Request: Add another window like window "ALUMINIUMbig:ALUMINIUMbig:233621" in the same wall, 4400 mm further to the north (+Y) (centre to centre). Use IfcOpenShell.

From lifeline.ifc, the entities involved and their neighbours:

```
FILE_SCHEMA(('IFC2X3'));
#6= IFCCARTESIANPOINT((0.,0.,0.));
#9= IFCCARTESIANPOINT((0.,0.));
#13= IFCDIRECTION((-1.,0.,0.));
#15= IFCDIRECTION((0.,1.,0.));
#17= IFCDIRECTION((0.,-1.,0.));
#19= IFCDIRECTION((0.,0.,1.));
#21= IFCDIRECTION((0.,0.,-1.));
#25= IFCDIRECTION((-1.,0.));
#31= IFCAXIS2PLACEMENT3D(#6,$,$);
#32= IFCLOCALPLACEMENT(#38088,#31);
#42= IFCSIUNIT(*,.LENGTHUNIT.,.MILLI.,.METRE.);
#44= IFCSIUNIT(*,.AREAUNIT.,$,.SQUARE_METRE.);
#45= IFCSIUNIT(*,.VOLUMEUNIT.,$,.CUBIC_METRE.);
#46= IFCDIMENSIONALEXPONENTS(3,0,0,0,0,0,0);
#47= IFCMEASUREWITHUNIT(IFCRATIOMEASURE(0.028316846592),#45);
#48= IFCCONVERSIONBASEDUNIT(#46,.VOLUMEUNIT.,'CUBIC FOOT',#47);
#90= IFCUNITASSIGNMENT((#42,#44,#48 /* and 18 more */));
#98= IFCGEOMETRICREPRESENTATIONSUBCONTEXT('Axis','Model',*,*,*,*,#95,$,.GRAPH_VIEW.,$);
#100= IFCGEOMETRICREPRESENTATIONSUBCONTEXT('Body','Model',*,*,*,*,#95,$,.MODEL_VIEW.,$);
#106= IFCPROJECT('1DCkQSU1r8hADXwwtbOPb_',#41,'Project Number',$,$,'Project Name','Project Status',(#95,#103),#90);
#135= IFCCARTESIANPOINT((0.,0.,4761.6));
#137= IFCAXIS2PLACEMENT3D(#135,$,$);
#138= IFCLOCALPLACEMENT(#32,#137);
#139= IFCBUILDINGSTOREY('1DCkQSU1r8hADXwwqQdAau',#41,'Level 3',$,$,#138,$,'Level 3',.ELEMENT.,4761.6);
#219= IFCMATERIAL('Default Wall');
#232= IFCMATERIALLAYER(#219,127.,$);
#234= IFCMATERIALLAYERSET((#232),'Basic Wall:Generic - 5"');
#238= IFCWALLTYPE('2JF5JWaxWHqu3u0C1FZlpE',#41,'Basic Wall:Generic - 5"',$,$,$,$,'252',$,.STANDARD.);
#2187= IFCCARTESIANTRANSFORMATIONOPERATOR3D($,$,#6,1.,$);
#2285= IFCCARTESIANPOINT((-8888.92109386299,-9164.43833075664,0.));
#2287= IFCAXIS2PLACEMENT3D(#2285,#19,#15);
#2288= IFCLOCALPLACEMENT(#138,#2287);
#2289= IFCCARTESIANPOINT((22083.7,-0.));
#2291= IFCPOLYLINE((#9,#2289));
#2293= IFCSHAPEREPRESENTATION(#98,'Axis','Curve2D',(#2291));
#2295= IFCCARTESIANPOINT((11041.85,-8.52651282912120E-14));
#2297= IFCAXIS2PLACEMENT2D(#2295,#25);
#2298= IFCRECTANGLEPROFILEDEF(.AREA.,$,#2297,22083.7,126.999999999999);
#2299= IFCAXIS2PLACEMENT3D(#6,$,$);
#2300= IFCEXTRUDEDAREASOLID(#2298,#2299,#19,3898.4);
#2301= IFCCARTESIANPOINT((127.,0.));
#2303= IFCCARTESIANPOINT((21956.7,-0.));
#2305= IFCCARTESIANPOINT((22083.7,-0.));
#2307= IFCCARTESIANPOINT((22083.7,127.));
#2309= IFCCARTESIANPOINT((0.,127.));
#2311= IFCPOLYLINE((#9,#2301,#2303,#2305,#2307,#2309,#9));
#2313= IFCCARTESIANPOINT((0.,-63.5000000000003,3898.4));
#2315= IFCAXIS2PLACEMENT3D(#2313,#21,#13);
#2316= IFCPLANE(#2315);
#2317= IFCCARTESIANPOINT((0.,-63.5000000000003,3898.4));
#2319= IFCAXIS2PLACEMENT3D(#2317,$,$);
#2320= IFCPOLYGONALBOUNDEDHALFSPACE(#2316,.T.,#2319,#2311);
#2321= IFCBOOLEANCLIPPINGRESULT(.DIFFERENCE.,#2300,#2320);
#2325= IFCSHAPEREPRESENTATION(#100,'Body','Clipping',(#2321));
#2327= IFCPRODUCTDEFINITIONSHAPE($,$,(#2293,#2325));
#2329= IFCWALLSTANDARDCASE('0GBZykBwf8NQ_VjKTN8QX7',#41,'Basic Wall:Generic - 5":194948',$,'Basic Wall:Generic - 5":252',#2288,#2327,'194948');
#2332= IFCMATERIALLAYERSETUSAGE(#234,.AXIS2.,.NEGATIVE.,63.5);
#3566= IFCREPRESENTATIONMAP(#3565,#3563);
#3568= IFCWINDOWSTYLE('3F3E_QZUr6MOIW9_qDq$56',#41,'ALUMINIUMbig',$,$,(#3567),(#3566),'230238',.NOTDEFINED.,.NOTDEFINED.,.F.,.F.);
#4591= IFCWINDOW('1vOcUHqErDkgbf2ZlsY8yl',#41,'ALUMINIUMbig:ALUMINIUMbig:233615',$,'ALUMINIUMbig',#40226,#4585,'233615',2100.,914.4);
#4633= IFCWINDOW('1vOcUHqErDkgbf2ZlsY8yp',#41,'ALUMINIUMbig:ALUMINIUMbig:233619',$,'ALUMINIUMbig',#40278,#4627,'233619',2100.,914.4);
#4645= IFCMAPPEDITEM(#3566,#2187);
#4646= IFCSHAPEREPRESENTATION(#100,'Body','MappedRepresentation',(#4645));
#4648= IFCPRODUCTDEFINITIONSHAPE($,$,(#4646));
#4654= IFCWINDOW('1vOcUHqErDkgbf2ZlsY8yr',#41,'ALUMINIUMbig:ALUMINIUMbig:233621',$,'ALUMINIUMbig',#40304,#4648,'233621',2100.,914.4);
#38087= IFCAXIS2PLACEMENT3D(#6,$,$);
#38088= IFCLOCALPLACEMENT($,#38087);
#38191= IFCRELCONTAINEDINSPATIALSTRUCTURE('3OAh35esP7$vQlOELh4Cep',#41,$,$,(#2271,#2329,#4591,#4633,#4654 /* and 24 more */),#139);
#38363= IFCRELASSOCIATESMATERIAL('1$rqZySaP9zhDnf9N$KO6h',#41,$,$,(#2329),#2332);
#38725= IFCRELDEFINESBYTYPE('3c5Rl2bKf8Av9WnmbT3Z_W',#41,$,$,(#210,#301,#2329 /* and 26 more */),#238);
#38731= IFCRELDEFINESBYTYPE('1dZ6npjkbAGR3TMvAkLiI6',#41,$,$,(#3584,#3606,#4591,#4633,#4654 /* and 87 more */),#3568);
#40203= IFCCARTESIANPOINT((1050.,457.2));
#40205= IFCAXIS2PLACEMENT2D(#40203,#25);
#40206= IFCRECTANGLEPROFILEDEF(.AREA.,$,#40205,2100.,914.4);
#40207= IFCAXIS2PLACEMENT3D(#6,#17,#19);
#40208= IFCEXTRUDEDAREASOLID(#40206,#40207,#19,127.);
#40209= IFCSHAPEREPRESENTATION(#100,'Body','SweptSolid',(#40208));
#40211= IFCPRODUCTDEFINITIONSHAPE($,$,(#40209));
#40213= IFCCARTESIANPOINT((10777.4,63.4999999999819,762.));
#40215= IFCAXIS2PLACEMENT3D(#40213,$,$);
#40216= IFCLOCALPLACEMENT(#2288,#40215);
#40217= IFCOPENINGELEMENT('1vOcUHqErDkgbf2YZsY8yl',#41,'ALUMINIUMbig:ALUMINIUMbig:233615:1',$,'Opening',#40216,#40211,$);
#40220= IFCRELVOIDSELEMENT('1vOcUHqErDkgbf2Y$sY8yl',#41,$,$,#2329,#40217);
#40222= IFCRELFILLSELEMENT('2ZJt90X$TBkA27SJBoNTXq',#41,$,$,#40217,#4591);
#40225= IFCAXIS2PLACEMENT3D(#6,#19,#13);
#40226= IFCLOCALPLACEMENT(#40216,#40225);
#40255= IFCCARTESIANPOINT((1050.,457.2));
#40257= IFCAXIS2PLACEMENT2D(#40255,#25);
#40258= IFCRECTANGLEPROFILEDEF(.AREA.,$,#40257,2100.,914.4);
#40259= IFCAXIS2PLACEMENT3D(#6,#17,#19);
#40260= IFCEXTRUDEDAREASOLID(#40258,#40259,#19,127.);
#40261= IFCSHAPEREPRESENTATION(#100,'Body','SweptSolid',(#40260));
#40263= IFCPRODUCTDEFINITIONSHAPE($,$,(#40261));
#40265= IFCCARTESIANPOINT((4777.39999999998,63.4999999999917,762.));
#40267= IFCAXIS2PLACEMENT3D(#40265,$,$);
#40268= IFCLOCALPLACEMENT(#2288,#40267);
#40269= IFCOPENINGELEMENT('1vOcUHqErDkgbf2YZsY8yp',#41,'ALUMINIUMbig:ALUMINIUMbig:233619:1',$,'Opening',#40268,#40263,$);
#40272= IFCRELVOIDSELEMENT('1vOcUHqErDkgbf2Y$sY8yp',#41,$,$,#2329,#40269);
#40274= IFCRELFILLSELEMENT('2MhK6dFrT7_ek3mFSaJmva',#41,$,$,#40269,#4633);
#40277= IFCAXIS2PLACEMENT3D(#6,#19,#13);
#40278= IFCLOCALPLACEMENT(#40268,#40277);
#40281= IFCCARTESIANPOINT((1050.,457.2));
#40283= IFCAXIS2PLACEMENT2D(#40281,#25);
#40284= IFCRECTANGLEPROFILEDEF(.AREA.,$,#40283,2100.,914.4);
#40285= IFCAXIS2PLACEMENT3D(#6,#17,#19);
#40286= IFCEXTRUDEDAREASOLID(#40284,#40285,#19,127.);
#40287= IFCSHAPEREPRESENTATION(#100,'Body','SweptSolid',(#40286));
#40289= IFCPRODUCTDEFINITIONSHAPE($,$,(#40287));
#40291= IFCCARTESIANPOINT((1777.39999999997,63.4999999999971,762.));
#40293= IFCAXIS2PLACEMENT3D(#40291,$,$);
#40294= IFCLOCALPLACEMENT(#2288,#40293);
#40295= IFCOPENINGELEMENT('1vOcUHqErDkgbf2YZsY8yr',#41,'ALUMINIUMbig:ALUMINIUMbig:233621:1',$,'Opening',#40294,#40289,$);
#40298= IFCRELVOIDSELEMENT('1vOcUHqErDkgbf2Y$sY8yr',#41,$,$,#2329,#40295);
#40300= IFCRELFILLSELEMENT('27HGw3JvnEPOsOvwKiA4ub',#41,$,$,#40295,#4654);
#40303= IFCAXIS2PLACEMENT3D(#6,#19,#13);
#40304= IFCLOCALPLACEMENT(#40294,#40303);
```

```python
import ifcopenshell
import ifcopenshell.api.feature
import ifcopenshell.api.geometry
import ifcopenshell.api.root
import ifcopenshell.geom
import ifcopenshell.util.element
import ifcopenshell.util.placement
import ifcopenshell.util.shape
import ifcopenshell.util.unit

model = ifcopenshell.open("lifeline.ifc")
unit_scale = ifcopenshell.util.unit.calculate_unit_scale(model)
settings = ifcopenshell.geom.settings()


def volume(element):
    """Net volume in cubic metres, openings subtracted."""
    shape = ifcopenshell.geom.create_shape(settings, element)
    return ifcopenshell.util.shape.get_volume(shape.geometry)


def reuse_history(source, copy):
    """copy_class also copies each property set's owner history, people and application; keep the originals."""
    for rel in copy.IsDefinedBy:
        if rel.is_a("IfcRelDefinesByProperties") and (history := rel.RelatingPropertyDefinition.OwnerHistory):
            rel.RelatingPropertyDefinition.OwnerHistory = source.OwnerHistory
            ifcopenshell.util.element.remove_deep2(model, history)


window = model.by_guid("1vOcUHqErDkgbf2ZlsY8yr")
opening = window.FillsVoids[0].RelatingOpeningElement
wall = opening.VoidsElements[0].RelatingBuildingElement
before = volume(wall)
shift = ifcopenshell.util.placement.get_local_placement(wall.ObjectPlacement)[:3, 0] * 4.4 / unit_scale

# copy_class copies the void relationship, type, container and properties, but no geometry.
new_opening = ifcopenshell.api.root.copy_class(model, product=opening)
new_opening.Representation = ifcopenshell.util.element.copy_deep(
    model, opening.Representation, exclude=["IfcGeometricRepresentationContext", "IfcRepresentationMap"]
)
new_opening.Name = "ALUMINIUMbig:ALUMINIUMbig"
new_window = ifcopenshell.api.root.copy_class(model, product=window)
new_window.Representation = ifcopenshell.util.element.copy_deep(
    model, window.Representation, exclude=["IfcGeometricRepresentationContext", "IfcRepresentationMap"]
)
new_window.Name = "ALUMINIUMbig:ALUMINIUMbig"
new_window.Tag = None
reuse_history(window, new_window)
fills = ifcopenshell.api.feature.add_filling(model, opening=new_opening, element=new_window)
fills.OwnerHistory = new_window.OwnerHistory  # required in IFC2X3

for old, new in ((opening, new_opening), (window, new_window)):
    matrix = ifcopenshell.util.placement.get_local_placement(old.ObjectPlacement)
    matrix[:3, 3] += shift
    ifcopenshell.api.geometry.edit_object_placement(model, product=new, matrix=matrix, is_si=False)

after = volume(wall)

print(f"wall volume {before:.3f} -> {after:.3f} m3")

model.write("lifeline_v2.ifc")
```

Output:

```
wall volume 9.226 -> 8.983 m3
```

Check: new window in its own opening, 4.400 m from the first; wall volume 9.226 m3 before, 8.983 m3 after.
